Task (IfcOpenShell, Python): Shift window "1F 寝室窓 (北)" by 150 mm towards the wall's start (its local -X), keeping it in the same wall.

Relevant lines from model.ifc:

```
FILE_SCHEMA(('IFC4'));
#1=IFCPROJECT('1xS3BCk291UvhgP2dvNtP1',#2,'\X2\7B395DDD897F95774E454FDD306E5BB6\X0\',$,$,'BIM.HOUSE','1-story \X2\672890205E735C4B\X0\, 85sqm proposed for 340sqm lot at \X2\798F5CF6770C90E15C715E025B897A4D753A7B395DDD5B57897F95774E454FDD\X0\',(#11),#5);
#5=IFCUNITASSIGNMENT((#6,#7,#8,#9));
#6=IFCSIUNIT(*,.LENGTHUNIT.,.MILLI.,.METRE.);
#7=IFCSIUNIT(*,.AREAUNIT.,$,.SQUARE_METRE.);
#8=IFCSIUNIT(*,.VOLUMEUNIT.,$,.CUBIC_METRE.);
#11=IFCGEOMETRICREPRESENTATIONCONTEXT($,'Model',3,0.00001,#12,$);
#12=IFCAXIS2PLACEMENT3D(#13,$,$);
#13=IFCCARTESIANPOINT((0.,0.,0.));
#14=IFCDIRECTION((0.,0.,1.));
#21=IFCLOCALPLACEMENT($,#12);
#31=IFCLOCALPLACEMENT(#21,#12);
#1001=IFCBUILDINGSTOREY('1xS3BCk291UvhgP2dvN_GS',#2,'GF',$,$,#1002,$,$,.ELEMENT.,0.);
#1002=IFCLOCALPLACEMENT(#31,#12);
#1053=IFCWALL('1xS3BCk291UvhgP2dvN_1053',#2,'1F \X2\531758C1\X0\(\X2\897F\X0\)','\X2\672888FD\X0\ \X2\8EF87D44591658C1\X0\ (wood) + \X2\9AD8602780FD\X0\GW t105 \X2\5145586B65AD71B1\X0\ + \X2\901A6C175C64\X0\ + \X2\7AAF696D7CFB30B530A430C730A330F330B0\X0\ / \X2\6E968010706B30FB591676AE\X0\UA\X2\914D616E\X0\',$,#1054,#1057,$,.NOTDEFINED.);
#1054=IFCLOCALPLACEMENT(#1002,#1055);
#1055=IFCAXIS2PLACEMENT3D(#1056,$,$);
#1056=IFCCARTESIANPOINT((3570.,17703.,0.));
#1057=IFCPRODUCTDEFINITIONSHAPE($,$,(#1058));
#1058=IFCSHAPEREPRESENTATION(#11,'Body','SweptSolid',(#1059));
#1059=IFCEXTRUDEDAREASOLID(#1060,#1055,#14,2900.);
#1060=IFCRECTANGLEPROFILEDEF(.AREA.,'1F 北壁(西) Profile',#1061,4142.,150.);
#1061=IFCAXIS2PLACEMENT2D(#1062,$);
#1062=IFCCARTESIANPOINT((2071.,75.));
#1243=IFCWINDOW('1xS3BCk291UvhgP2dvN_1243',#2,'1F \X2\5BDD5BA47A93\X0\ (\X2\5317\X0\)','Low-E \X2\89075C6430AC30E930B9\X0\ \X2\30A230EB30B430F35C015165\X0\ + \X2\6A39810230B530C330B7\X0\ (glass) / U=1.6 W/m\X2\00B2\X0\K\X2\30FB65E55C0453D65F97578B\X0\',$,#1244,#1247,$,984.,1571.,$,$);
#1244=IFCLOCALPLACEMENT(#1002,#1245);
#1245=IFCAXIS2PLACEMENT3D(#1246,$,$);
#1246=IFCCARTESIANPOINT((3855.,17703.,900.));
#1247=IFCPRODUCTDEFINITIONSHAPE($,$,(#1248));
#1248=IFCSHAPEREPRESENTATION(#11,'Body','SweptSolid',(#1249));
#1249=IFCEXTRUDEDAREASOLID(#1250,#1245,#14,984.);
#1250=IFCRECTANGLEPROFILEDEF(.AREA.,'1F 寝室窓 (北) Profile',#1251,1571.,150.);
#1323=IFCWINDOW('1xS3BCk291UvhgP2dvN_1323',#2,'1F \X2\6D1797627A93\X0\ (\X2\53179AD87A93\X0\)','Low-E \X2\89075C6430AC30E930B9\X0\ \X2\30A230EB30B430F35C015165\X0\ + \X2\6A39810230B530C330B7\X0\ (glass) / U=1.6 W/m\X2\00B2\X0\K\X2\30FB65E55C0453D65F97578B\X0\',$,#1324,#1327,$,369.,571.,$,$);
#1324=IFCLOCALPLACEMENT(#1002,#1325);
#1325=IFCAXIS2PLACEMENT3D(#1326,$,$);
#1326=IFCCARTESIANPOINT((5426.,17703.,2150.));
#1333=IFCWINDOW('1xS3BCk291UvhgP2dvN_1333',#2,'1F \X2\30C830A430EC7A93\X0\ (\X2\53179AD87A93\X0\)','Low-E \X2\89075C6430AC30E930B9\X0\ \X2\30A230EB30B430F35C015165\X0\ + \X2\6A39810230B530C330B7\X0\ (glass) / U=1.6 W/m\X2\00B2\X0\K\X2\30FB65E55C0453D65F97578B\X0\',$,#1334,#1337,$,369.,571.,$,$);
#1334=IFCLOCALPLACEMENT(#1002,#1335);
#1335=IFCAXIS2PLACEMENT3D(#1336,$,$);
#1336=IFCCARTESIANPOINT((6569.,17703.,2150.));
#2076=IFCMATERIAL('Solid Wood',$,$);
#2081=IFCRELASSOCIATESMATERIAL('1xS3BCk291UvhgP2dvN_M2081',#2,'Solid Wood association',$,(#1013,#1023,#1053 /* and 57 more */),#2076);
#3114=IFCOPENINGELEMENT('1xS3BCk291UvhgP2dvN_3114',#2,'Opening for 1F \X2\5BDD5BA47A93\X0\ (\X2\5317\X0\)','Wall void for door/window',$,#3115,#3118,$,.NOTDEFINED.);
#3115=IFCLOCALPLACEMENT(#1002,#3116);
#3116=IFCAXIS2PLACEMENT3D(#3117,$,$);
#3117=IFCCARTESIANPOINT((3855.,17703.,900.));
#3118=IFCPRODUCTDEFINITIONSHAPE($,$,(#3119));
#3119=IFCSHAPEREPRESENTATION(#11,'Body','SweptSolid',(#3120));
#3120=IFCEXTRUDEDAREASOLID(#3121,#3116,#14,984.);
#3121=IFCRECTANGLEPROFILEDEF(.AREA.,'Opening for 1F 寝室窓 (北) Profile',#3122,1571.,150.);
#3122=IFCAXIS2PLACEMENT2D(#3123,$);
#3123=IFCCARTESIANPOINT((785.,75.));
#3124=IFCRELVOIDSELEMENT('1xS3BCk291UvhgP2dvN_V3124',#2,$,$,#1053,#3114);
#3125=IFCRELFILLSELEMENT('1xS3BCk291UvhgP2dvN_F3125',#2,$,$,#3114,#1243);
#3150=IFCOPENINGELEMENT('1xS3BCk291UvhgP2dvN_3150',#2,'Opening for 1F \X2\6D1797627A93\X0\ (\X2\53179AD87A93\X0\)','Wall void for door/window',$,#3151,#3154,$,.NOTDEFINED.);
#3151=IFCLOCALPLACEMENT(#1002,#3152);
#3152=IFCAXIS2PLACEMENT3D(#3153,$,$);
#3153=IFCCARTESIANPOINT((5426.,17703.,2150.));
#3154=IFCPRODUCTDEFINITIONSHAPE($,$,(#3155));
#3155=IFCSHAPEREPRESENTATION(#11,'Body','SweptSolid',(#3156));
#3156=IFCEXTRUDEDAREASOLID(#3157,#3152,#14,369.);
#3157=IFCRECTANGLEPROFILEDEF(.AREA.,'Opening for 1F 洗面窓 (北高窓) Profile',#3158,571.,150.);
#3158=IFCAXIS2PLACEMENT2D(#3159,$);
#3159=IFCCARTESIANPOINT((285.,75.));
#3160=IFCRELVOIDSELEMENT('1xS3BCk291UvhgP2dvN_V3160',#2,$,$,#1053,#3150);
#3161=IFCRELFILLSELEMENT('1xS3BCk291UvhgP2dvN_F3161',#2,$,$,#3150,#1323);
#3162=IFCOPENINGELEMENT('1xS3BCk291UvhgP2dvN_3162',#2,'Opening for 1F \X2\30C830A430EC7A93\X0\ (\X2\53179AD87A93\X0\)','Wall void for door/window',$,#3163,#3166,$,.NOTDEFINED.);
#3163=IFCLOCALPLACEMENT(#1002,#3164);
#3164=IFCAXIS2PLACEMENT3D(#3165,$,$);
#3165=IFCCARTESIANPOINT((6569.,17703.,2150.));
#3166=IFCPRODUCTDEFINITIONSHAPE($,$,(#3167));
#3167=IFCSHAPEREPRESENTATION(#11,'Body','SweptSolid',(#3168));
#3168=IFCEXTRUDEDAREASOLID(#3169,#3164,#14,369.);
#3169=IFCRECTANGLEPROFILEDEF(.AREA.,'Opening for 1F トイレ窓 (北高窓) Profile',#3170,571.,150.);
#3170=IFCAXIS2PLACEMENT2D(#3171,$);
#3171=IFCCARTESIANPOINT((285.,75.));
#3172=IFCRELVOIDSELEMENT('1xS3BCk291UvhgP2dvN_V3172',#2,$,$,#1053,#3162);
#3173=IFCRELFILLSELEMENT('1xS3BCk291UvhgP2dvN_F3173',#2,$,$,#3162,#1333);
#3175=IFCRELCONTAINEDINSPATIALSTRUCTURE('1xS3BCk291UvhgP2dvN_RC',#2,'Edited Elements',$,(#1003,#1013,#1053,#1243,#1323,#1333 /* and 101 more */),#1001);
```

```python
import ifcopenshell
import ifcopenshell.api.geometry
import ifcopenshell.util.placement
import ifcopenshell.util.unit

model = ifcopenshell.open("model.ifc")
unit_scale = ifcopenshell.util.unit.calculate_unit_scale(model)

window = model.by_guid("1xS3BCk291UvhgP2dvN_1243")
opening = window.FillsVoids[0].RelatingOpeningElement
wall = opening.VoidsElements[0].RelatingBuildingElement

wall_matrix = ifcopenshell.util.placement.get_local_placement(wall.ObjectPlacement)
shift = wall_matrix[:3, 0] * -0.15 / unit_scale
before = ifcopenshell.util.placement.get_local_placement(window.ObjectPlacement)[:3, 3].copy()

# The window is not placed relative to its opening, so move both.
for product in (opening, window):
    matrix = ifcopenshell.util.placement.get_local_placement(product.ObjectPlacement)
    matrix[:3, 3] += shift
    ifcopenshell.api.geometry.edit_object_placement(model, product=product, matrix=matrix, is_si=False)

after = ifcopenshell.util.placement.get_local_placement(window.ObjectPlacement)[:3, 3]
print("window moved by", (after - before).round(3) + 0.0)

model.write("model_v2.ifc")
```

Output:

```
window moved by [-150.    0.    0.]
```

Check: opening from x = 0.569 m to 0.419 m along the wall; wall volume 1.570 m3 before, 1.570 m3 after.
